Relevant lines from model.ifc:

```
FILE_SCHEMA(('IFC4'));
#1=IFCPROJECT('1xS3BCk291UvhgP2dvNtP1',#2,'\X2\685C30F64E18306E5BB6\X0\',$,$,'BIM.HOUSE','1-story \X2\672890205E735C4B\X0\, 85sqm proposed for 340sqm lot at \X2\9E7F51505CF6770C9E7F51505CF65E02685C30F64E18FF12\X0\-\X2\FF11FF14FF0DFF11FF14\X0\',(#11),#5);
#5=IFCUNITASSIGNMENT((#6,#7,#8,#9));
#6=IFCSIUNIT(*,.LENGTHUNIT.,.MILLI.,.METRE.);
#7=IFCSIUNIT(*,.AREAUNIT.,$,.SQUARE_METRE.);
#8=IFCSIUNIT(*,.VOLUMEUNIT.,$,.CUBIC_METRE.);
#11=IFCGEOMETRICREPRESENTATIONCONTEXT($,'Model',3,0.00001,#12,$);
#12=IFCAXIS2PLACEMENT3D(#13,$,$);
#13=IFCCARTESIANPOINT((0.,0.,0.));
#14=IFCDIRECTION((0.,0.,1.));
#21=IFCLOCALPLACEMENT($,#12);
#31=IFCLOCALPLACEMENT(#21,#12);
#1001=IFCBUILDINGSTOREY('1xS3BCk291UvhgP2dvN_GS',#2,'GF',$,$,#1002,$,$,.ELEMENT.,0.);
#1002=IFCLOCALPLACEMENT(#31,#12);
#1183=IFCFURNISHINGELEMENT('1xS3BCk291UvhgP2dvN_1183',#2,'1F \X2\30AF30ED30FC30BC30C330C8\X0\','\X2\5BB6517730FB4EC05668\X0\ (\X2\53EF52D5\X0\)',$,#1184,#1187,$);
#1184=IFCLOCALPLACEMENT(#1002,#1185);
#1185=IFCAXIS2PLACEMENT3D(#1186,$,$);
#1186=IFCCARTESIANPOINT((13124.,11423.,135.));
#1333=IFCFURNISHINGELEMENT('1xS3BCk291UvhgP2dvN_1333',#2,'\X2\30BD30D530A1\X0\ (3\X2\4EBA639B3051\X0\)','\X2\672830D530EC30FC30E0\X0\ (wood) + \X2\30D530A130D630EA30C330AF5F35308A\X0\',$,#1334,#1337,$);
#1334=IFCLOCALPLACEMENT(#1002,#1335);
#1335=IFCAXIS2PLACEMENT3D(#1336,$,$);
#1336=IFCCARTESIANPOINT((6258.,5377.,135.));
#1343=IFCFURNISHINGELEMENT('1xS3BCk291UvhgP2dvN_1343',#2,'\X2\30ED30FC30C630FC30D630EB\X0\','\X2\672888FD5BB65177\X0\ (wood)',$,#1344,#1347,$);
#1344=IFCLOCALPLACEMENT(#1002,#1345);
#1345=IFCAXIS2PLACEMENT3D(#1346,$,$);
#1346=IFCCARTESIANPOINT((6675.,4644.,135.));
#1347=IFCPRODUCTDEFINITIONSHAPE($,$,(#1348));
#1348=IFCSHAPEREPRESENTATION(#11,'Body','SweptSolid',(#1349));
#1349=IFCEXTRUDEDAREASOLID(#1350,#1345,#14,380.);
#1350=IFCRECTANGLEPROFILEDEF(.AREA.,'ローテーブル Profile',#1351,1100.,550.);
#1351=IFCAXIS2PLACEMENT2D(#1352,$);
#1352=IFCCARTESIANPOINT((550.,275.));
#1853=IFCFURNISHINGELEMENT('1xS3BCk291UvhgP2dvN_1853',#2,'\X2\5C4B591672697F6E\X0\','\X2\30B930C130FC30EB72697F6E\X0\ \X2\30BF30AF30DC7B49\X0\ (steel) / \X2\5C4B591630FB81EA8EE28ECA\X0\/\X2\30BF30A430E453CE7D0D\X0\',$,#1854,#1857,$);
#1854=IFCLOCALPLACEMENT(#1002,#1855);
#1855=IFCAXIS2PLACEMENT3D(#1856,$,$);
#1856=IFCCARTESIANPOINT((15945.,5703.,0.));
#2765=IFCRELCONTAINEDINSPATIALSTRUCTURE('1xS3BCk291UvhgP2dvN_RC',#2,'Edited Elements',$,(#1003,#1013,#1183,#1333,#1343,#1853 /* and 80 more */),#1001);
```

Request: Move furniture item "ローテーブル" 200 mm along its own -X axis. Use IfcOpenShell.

```python
import ifcopenshell
import ifcopenshell.api.geometry
import ifcopenshell.util.placement

model = ifcopenshell.open("model.ifc")

item = model.by_guid("1xS3BCk291UvhgP2dvN_1343")
matrix = ifcopenshell.util.placement.get_local_placement(item.ObjectPlacement)
matrix[:3, 3] -= matrix[:3, 0] * 200.0
ifcopenshell.api.geometry.edit_object_placement(model, product=item, matrix=matrix, is_si=False)

print(ifcopenshell.util.placement.get_local_placement(item.ObjectPlacement).round(3) + 0.0)

model.write("model_edited.ifc")
```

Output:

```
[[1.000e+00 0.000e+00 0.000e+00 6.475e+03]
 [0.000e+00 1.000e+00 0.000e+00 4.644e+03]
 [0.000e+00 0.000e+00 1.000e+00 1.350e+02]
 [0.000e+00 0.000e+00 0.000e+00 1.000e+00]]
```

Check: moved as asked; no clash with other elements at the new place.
